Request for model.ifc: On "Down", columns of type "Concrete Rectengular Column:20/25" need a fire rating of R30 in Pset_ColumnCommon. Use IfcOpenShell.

First a look at what the model holds.

```python
import ifcopenshell
import ifcopenshell.util.element

model = ifcopenshell.open("model.ifc")
print(model.schema)
storey = next(s for s in model.by_type("IfcBuildingStorey") if s.Name == "Down")
columns = [e for e in ifcopenshell.util.element.get_decomposition(storey) if e.is_a("IfcColumn")]
seen = {}
for e in columns:
    element_type = ifcopenshell.util.element.get_type(e)
    key = (element_type.Name if element_type != e and element_type else None, ifcopenshell.util.element.get_pset(e, "Pset_ColumnCommon", "FireRating"))
    seen[key] = seen.get(key, 0) + 1
for (name, value), count in sorted(seen.items(), key=str):
    print(count, "x", name, "|", value)
```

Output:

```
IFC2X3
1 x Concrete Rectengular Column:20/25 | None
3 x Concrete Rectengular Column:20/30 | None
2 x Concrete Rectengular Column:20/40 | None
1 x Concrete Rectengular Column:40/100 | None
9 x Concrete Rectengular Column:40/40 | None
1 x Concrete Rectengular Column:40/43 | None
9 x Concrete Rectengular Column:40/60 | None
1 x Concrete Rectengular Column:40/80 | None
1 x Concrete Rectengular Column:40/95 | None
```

```python
import ifcopenshell
import ifcopenshell.api.pset
import ifcopenshell.util.element

model = ifcopenshell.open("model.ifc")

storey = next(s for s in model.by_type("IfcBuildingStorey") if s.Name == "Down")
columns = [e for e in ifcopenshell.util.element.get_decomposition(storey) if e.is_a("IfcColumn")]

count = 0
for e in columns:
    element_type = ifcopenshell.util.element.get_type(e)
    if element_type in (None, e) or element_type.Name != "Concrete Rectengular Column:20/25":
        continue
    # add_pset returns the element's existing set when there is one.
    pset = ifcopenshell.api.pset.add_pset(model, product=e, name="Pset_ColumnCommon")
    ifcopenshell.api.pset.edit_pset(model, pset=pset, properties={"FireRating": "R30"})
    count += 1

print(count, "columns updated")

model.write("model_rev.ifc")
```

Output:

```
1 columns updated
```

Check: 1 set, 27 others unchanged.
